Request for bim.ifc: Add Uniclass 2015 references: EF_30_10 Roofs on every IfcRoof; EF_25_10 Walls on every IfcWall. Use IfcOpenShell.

First a look at what the model holds.

```python
import ifcopenshell

model = ifcopenshell.open("bim.ifc")
print(model.schema)
print("classifications:", [c.Name for c in model.by_type("IfcClassification")])
for ifc_class in ("IfcDoor", "IfcRoof", "IfcStair", "IfcWall", "IfcWindow"):
    print(ifc_class, len(model.by_type(ifc_class)))
```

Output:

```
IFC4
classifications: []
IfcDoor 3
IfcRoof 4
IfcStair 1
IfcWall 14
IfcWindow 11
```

```python
import ifcopenshell
import ifcopenshell.api.classification

model = ifcopenshell.open("bim.ifc")

system = ifcopenshell.api.classification.add_classification(model, classification="Uniclass 2015")

codes = {
    "IfcRoof": ("EF_30_10", "Roofs"),
    "IfcWall": ("EF_25_10", "Walls"),
}
for ifc_class, (code, name) in codes.items():
    products = model.by_type(ifc_class)
    ifcopenshell.api.classification.add_reference(
        model, products=products, classification=system, identification=code, name=name
    )
    print(code, len(products))

model.write("bim_v2.ifc")
```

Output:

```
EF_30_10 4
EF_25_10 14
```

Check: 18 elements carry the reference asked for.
